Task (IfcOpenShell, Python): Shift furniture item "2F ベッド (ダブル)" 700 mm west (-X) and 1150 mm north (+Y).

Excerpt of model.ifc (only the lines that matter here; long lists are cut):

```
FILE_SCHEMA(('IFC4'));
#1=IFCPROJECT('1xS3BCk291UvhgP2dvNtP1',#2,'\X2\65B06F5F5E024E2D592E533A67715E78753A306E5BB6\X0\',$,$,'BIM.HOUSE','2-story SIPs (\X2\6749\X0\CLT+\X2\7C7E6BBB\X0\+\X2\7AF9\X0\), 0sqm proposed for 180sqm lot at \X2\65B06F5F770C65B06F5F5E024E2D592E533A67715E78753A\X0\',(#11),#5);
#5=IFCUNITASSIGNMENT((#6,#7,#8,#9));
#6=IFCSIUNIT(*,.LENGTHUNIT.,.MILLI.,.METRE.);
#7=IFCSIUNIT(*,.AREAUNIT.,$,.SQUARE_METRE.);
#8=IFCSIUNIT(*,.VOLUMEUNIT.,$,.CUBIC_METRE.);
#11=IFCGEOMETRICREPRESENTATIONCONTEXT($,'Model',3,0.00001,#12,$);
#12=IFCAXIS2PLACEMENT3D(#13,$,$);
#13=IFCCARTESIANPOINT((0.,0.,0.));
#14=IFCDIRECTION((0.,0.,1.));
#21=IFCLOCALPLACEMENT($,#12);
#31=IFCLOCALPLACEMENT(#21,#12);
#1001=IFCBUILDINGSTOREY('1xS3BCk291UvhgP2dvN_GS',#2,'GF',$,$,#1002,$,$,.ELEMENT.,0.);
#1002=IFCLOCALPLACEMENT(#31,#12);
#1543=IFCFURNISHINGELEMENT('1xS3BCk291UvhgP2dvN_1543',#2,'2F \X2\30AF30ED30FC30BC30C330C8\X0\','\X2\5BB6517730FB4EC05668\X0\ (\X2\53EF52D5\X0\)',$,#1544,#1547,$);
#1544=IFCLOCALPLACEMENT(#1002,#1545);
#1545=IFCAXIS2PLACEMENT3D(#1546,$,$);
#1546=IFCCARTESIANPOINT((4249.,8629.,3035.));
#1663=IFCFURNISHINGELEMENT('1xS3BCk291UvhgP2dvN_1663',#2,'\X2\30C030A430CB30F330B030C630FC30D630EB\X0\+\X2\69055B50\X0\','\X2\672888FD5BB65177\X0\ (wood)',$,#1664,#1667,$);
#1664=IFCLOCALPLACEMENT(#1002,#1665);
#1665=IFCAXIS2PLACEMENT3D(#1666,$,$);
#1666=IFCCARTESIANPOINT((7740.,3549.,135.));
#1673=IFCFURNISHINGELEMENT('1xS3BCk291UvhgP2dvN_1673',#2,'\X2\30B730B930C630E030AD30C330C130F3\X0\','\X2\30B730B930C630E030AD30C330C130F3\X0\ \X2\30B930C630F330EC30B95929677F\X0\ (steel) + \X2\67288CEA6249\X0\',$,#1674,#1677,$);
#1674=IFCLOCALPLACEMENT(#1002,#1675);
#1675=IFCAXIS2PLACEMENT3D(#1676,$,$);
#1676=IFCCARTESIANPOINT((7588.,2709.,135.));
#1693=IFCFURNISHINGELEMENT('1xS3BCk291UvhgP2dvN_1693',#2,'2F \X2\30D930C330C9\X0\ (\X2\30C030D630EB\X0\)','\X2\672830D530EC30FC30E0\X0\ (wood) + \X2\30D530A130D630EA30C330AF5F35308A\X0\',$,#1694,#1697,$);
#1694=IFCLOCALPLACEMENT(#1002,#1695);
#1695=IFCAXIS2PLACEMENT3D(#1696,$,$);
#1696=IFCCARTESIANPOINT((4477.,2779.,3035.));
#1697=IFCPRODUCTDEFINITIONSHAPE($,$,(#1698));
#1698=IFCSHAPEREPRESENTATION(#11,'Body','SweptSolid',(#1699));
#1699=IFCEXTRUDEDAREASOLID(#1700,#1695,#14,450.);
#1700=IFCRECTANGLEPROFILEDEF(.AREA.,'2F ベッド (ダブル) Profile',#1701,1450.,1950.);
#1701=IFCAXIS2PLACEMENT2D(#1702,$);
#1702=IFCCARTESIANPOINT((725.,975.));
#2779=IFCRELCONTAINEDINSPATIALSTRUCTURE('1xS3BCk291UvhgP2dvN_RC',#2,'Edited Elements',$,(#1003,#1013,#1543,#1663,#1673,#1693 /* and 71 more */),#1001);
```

```python
import ifcopenshell
import ifcopenshell.api.geometry
import ifcopenshell.util.placement
import ifcopenshell.util.unit

model = ifcopenshell.open("model.ifc")
unit_scale = ifcopenshell.util.unit.calculate_unit_scale(model)

item = model.by_guid("1xS3BCk291UvhgP2dvN_1693")
matrix = ifcopenshell.util.placement.get_local_placement(item.ObjectPlacement)
matrix[0, 3] -= 0.7 / unit_scale
matrix[1, 3] += 1.15 / unit_scale
ifcopenshell.api.geometry.edit_object_placement(model, product=item, matrix=matrix, is_si=False)

print(ifcopenshell.util.placement.get_local_placement(item.ObjectPlacement).round(3) + 0.0)

model.write("model_rev.ifc")
```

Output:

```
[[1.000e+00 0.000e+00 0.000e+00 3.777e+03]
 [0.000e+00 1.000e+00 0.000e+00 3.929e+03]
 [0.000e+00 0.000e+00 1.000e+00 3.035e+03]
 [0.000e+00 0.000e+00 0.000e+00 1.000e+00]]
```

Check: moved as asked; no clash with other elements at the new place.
